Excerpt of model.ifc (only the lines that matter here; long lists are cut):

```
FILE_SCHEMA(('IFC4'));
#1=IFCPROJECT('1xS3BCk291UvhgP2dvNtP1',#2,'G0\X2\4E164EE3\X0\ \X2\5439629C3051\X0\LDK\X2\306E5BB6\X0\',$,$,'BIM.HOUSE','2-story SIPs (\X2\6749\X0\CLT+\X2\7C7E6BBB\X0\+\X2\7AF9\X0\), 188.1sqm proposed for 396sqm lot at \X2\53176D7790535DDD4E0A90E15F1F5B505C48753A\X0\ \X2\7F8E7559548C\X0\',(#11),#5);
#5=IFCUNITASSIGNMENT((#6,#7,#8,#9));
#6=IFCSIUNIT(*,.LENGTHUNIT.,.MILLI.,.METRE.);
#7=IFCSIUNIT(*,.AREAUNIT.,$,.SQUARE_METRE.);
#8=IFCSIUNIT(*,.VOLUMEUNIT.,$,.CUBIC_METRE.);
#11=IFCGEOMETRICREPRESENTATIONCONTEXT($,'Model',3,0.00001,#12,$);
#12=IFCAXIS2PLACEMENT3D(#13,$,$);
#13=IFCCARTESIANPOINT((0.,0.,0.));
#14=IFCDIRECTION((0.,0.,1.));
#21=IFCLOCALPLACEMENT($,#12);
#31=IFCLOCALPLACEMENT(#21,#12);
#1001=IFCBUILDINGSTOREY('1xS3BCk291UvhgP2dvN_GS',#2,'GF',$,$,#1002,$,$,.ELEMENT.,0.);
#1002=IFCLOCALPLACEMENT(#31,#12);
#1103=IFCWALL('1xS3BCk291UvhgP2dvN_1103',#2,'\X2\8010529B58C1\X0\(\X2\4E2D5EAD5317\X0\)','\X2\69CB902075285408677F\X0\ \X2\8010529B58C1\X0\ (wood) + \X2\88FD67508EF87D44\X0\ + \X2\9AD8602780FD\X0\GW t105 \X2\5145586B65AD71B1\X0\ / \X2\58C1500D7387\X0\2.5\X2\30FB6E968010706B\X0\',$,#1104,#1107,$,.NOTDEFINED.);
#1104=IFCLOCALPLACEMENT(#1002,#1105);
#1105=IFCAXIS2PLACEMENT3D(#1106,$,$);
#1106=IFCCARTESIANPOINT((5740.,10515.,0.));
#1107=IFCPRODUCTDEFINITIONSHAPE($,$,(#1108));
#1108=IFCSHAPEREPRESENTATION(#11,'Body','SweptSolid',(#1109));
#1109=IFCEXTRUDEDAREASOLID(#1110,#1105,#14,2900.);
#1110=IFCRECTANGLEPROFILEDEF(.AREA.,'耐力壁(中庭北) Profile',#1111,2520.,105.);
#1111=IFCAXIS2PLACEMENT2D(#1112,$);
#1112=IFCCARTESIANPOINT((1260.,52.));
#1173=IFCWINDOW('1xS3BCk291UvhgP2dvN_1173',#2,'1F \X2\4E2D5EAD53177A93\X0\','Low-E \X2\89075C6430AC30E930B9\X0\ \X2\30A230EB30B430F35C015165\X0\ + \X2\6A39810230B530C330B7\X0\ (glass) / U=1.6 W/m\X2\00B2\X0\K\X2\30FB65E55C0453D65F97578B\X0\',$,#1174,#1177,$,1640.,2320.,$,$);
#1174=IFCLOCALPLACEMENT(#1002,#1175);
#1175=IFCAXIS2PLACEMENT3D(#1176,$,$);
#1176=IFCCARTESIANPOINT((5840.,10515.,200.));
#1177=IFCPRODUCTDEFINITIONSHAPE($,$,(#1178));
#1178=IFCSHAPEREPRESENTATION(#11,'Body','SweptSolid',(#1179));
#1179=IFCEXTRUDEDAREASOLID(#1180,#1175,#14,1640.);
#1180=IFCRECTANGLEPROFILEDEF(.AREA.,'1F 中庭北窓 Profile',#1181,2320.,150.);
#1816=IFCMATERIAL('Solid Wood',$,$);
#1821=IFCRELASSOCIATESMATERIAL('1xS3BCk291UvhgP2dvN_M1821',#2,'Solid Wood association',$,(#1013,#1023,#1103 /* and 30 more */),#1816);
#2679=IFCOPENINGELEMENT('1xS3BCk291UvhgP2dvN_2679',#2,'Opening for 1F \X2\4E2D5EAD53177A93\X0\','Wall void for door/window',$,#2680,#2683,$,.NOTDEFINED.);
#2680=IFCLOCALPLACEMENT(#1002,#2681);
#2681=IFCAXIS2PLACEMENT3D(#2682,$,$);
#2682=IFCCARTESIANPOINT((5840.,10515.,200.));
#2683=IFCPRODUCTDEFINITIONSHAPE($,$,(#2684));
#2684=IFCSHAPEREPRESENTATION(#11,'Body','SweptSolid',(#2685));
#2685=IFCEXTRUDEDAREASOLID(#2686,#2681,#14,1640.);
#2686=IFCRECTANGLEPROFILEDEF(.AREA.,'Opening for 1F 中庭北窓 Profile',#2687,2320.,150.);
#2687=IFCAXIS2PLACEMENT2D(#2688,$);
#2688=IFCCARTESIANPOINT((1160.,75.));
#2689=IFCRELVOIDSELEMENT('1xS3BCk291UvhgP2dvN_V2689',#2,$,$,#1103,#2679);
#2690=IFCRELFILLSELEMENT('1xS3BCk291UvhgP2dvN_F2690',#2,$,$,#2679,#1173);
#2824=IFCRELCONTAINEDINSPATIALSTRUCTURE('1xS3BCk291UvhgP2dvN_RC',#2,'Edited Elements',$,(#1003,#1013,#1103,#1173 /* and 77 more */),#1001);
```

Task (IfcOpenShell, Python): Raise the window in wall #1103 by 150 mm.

```python
import numpy as np
import ifcopenshell
import ifcopenshell.api.geometry
import ifcopenshell.util.placement
import ifcopenshell.util.unit

model = ifcopenshell.open("model.ifc")
unit_scale = ifcopenshell.util.unit.calculate_unit_scale(model)

window = model.by_guid("1xS3BCk291UvhgP2dvN_1173")
opening = window.FillsVoids[0].RelatingOpeningElement
dz = 0.15 / unit_scale

shift = np.array([0.0, 0.0, dz])
# The window is not placed relative to its opening, so move both.
for product in (opening, window):
    matrix = ifcopenshell.util.placement.get_local_placement(product.ObjectPlacement)
    matrix[:3, 3] += shift
    ifcopenshell.api.geometry.edit_object_placement(model, product=product, matrix=matrix, is_si=False)

print(f"moved by {dz * unit_scale:+.3f} m")

model.write("model_v2.ifc")
```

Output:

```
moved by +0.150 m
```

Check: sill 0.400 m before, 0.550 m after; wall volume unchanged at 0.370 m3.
